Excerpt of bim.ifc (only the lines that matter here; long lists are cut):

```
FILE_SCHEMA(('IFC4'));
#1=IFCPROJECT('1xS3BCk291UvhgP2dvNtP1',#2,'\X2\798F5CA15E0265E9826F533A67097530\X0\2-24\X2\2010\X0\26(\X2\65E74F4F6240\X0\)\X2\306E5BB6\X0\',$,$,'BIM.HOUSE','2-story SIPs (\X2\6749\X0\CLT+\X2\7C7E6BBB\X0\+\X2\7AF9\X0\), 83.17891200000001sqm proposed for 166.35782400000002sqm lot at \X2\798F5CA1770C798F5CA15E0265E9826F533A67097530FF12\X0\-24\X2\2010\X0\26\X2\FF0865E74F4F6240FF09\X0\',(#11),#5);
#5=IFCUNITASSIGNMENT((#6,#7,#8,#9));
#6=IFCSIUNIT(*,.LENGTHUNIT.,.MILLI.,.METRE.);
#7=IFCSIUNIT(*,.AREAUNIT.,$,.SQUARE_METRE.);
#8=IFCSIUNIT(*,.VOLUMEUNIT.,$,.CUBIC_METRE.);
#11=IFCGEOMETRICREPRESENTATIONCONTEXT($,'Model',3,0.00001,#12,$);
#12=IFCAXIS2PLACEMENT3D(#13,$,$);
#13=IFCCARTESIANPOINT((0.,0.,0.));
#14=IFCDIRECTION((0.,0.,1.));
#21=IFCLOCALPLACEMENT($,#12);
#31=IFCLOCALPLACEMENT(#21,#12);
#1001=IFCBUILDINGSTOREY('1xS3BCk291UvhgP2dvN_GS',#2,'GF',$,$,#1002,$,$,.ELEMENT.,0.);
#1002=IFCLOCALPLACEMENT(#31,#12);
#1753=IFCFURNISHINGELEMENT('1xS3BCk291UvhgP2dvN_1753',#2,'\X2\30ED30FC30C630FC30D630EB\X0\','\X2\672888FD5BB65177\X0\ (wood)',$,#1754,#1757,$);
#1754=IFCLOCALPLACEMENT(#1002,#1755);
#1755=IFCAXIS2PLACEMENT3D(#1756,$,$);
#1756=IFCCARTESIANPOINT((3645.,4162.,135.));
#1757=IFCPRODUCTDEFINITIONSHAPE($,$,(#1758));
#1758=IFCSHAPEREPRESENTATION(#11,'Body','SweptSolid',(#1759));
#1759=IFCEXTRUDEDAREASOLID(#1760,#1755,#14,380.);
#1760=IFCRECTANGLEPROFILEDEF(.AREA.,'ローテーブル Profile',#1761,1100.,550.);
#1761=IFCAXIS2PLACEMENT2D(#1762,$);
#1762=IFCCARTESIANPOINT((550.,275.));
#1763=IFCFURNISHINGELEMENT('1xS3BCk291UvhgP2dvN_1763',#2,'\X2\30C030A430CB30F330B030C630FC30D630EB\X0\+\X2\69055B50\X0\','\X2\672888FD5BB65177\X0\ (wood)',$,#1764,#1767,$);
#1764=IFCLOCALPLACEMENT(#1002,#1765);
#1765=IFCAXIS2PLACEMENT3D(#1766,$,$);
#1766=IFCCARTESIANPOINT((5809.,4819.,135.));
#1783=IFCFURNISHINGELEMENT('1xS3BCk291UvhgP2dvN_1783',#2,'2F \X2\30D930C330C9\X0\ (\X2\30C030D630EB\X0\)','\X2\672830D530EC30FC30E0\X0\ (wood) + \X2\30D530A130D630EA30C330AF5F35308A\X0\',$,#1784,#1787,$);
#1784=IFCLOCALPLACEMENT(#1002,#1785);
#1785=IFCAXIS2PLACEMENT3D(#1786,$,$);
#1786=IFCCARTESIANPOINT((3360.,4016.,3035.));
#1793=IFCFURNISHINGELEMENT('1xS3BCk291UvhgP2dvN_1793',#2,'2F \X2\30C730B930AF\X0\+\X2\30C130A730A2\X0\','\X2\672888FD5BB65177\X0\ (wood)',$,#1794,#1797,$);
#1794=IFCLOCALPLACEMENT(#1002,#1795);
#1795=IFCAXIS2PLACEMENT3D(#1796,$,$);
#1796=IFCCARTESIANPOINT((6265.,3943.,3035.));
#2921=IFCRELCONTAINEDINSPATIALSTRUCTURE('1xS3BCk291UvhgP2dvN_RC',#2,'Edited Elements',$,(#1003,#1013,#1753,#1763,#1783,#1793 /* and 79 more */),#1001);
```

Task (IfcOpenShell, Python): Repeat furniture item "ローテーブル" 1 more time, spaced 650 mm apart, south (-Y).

```python
import numpy as np
import ifcopenshell
import ifcopenshell.api.geometry
import ifcopenshell.api.root
import ifcopenshell.util.element
import ifcopenshell.util.placement

model = ifcopenshell.open("bim.ifc")


def reuse_history(source, copy):
    """copy_class also copies each property set's owner history, people and application; keep the originals."""
    for rel in copy.IsDefinedBy:
        if rel.is_a("IfcRelDefinesByProperties") and (history := rel.RelatingPropertyDefinition.OwnerHistory):
            rel.RelatingPropertyDefinition.OwnerHistory = source.OwnerHistory
            ifcopenshell.util.element.remove_deep2(model, history)


source = model.by_guid("1xS3BCk291UvhgP2dvN_1753")
base = ifcopenshell.util.placement.get_local_placement(source.ObjectPlacement)
step = np.array([0.0, -1.0, 0.0]) * 650.0

for i in range(1, 2):
    copy = ifcopenshell.api.root.copy_class(model, product=source)
    copy.Representation = ifcopenshell.util.element.copy_deep(
        model, source.Representation, exclude=["IfcGeometricRepresentationContext", "IfcRepresentationMap"]
    )
    reuse_history(source, copy)
    matrix = base.copy()
    matrix[:3, 3] += i * step
    print("added at", matrix[:3, 3].round(3) + 0.0)
    ifcopenshell.api.geometry.edit_object_placement(model, product=copy, matrix=matrix, is_si=False)

model.write("bim_updated.ifc")
```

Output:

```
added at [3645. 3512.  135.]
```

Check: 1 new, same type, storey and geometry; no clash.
